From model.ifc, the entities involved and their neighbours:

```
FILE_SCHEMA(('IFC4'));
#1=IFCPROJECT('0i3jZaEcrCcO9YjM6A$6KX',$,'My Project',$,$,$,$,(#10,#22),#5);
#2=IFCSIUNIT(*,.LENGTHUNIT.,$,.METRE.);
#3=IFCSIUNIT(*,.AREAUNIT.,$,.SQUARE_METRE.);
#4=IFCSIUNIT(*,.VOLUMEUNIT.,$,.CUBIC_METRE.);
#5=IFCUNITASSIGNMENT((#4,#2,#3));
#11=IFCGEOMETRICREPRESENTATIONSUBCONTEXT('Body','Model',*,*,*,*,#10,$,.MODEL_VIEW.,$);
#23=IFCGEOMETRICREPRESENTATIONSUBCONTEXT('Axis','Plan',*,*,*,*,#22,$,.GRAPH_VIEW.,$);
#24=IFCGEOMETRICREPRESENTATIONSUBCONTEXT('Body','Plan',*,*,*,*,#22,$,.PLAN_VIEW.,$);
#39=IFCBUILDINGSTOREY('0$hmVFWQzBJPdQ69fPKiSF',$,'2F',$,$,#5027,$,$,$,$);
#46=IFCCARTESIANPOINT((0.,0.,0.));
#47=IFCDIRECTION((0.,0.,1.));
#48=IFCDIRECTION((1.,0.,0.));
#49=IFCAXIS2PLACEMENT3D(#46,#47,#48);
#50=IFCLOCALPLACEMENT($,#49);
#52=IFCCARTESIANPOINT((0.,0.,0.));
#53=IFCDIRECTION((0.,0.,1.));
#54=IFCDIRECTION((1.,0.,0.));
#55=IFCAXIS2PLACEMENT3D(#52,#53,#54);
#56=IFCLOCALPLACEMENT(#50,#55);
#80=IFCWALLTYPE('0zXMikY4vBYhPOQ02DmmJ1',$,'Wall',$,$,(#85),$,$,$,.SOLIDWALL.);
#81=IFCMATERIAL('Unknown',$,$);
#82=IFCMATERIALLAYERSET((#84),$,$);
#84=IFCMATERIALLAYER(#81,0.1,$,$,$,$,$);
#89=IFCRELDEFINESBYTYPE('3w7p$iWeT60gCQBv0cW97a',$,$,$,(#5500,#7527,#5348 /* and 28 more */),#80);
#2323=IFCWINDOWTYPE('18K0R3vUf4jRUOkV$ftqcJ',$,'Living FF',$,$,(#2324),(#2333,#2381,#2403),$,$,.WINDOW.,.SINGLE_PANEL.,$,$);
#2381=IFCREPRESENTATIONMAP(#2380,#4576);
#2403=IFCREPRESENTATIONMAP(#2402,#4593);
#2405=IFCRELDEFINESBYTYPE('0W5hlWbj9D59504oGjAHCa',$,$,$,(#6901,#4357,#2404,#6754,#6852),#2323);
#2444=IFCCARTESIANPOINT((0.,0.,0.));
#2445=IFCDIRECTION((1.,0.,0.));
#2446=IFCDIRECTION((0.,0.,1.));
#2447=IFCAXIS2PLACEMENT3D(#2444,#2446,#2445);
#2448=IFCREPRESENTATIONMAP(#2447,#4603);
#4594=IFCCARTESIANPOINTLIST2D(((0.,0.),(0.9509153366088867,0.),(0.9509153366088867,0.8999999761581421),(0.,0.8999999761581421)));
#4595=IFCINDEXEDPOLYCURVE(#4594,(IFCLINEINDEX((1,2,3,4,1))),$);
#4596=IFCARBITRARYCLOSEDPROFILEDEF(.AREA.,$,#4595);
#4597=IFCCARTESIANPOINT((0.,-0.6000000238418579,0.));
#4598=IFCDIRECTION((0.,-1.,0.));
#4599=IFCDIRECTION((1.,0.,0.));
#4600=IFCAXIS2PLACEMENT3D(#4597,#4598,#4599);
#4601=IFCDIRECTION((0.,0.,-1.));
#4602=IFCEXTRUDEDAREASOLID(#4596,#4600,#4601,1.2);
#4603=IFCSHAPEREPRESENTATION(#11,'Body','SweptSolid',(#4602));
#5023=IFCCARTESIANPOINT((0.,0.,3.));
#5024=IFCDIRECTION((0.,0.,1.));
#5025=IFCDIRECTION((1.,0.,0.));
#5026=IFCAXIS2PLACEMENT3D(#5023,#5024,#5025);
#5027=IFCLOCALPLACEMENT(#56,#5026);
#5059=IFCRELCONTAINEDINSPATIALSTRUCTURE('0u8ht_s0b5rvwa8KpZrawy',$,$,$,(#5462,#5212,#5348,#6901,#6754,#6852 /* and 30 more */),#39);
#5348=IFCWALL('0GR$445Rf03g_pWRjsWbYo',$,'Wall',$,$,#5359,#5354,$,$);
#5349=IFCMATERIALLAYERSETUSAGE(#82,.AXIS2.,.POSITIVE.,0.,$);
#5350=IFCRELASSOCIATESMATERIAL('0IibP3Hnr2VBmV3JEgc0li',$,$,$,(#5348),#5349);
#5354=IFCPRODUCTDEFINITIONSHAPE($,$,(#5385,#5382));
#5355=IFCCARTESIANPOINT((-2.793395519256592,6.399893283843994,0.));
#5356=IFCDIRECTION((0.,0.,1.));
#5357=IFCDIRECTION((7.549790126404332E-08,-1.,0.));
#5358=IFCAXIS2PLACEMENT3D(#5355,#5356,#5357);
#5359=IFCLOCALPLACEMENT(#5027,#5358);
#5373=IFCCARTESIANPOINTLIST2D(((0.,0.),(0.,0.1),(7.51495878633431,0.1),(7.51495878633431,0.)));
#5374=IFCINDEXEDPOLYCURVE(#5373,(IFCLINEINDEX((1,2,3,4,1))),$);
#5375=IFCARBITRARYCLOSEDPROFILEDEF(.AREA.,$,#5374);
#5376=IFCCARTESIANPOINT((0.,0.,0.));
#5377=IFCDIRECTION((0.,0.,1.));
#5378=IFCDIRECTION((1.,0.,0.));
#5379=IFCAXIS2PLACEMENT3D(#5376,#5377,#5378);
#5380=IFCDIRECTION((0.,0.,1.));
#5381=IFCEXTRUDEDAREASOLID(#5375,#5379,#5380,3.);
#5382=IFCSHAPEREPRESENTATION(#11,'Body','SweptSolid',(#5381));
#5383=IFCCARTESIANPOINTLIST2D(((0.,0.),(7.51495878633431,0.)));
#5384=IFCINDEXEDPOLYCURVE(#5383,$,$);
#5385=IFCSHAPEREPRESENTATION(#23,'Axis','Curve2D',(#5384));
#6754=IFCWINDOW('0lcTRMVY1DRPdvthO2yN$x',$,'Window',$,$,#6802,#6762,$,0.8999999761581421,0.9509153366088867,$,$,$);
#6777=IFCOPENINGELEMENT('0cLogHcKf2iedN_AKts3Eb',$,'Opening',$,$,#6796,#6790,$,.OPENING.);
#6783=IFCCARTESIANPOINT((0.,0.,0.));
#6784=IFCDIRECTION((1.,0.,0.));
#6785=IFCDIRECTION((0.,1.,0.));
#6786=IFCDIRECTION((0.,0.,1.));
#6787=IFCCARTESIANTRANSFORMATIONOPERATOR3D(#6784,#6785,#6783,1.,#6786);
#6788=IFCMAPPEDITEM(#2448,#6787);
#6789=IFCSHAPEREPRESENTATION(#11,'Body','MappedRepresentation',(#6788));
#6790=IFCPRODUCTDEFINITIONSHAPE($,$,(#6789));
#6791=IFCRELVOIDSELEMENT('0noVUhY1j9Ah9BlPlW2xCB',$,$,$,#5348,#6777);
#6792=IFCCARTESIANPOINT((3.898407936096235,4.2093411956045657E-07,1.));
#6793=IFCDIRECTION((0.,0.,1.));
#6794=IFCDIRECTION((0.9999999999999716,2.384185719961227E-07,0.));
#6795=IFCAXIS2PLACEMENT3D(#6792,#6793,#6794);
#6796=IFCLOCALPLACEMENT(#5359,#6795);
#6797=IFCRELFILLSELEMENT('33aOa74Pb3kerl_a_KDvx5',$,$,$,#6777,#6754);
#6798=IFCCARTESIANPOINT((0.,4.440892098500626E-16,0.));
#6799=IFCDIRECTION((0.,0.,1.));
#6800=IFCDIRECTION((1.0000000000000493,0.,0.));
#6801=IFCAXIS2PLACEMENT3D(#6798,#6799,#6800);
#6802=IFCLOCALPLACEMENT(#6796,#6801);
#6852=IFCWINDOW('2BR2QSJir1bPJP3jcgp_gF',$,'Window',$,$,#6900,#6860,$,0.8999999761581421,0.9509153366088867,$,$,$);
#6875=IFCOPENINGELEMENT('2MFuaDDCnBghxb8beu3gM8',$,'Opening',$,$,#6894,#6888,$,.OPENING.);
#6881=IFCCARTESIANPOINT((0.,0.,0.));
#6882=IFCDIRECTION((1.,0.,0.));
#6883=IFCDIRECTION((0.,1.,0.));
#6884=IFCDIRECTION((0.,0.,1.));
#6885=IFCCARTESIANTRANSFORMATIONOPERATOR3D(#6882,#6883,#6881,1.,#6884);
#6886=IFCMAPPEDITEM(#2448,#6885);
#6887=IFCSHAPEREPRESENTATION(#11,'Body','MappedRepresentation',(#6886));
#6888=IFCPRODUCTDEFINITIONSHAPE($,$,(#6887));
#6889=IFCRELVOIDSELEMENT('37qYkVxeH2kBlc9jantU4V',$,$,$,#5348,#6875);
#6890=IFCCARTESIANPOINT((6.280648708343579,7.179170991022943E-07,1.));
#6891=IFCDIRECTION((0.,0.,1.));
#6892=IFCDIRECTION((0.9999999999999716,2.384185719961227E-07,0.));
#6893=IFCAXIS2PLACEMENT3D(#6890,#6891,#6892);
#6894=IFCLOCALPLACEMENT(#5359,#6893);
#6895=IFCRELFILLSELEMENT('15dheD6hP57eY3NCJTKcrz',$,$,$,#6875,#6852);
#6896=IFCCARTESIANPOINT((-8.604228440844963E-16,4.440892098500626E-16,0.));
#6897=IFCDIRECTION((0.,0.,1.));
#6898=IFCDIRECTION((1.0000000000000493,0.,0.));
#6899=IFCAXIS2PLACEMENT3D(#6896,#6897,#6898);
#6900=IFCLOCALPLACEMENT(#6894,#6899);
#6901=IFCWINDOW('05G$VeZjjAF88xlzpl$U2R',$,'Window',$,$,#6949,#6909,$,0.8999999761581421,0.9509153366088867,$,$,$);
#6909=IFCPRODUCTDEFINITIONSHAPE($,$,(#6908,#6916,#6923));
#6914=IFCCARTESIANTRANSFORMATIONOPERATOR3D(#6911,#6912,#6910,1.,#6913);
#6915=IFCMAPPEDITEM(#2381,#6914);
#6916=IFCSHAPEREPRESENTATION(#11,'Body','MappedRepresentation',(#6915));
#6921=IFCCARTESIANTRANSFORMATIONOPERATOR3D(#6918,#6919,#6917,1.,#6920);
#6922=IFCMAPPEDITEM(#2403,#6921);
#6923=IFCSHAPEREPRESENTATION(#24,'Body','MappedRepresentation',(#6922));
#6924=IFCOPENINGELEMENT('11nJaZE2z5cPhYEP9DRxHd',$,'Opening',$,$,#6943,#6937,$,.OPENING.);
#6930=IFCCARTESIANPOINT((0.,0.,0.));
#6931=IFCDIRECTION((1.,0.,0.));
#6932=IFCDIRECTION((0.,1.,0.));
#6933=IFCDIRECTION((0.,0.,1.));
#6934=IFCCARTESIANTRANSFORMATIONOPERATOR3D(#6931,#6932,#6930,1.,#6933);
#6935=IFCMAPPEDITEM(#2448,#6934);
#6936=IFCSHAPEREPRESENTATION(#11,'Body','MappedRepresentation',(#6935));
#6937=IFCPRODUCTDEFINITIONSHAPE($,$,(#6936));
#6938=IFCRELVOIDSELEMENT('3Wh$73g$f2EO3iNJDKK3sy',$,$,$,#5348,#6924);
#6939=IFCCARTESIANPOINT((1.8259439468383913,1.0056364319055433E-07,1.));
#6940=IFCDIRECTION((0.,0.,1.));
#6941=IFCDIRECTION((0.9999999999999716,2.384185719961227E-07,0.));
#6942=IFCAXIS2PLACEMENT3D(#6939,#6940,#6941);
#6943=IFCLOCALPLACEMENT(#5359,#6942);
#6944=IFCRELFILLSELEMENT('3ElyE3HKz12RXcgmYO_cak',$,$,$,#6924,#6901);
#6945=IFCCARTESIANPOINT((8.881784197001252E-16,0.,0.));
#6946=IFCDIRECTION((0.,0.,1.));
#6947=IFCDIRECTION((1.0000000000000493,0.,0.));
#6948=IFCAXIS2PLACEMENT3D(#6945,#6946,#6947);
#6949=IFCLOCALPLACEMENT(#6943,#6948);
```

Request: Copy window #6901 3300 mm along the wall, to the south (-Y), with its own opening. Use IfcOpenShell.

```python
import ifcopenshell
import ifcopenshell.api.feature
import ifcopenshell.api.geometry
import ifcopenshell.api.root
import ifcopenshell.geom
import ifcopenshell.util.element
import ifcopenshell.util.placement
import ifcopenshell.util.shape
import ifcopenshell.util.unit

model = ifcopenshell.open("model.ifc")
unit_scale = ifcopenshell.util.unit.calculate_unit_scale(model)
settings = ifcopenshell.geom.settings()


def volume(element):
    """Net volume in cubic metres, openings subtracted."""
    shape = ifcopenshell.geom.create_shape(settings, element)
    return ifcopenshell.util.shape.get_volume(shape.geometry)


window = model.by_id(6901)
opening = window.FillsVoids[0].RelatingOpeningElement
wall = opening.VoidsElements[0].RelatingBuildingElement
before = volume(wall)
shift = ifcopenshell.util.placement.get_local_placement(wall.ObjectPlacement)[:3, 0] * 3.3 / unit_scale

# copy_class copies the void relationship, type, container and properties, but no geometry.
new_opening = ifcopenshell.api.root.copy_class(model, product=opening)
new_opening.Representation = ifcopenshell.util.element.copy_deep(
    model, opening.Representation, exclude=["IfcGeometricRepresentationContext", "IfcRepresentationMap"]
)
new_window = ifcopenshell.api.root.copy_class(model, product=window)
new_window.Representation = ifcopenshell.util.element.copy_deep(
    model, window.Representation, exclude=["IfcGeometricRepresentationContext", "IfcRepresentationMap"]
)
ifcopenshell.api.feature.add_filling(model, opening=new_opening, element=new_window)

for old, new in ((opening, new_opening), (window, new_window)):
    matrix = ifcopenshell.util.placement.get_local_placement(old.ObjectPlacement)
    matrix[:3, 3] += shift
    ifcopenshell.api.geometry.edit_object_placement(model, product=new, matrix=matrix, is_si=False)

after = volume(wall)

print(f"wall volume {before:.3f} -> {after:.3f} m3")

model.write("model_edited.ifc")
```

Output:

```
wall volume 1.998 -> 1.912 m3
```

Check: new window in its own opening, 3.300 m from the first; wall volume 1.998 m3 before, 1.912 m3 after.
